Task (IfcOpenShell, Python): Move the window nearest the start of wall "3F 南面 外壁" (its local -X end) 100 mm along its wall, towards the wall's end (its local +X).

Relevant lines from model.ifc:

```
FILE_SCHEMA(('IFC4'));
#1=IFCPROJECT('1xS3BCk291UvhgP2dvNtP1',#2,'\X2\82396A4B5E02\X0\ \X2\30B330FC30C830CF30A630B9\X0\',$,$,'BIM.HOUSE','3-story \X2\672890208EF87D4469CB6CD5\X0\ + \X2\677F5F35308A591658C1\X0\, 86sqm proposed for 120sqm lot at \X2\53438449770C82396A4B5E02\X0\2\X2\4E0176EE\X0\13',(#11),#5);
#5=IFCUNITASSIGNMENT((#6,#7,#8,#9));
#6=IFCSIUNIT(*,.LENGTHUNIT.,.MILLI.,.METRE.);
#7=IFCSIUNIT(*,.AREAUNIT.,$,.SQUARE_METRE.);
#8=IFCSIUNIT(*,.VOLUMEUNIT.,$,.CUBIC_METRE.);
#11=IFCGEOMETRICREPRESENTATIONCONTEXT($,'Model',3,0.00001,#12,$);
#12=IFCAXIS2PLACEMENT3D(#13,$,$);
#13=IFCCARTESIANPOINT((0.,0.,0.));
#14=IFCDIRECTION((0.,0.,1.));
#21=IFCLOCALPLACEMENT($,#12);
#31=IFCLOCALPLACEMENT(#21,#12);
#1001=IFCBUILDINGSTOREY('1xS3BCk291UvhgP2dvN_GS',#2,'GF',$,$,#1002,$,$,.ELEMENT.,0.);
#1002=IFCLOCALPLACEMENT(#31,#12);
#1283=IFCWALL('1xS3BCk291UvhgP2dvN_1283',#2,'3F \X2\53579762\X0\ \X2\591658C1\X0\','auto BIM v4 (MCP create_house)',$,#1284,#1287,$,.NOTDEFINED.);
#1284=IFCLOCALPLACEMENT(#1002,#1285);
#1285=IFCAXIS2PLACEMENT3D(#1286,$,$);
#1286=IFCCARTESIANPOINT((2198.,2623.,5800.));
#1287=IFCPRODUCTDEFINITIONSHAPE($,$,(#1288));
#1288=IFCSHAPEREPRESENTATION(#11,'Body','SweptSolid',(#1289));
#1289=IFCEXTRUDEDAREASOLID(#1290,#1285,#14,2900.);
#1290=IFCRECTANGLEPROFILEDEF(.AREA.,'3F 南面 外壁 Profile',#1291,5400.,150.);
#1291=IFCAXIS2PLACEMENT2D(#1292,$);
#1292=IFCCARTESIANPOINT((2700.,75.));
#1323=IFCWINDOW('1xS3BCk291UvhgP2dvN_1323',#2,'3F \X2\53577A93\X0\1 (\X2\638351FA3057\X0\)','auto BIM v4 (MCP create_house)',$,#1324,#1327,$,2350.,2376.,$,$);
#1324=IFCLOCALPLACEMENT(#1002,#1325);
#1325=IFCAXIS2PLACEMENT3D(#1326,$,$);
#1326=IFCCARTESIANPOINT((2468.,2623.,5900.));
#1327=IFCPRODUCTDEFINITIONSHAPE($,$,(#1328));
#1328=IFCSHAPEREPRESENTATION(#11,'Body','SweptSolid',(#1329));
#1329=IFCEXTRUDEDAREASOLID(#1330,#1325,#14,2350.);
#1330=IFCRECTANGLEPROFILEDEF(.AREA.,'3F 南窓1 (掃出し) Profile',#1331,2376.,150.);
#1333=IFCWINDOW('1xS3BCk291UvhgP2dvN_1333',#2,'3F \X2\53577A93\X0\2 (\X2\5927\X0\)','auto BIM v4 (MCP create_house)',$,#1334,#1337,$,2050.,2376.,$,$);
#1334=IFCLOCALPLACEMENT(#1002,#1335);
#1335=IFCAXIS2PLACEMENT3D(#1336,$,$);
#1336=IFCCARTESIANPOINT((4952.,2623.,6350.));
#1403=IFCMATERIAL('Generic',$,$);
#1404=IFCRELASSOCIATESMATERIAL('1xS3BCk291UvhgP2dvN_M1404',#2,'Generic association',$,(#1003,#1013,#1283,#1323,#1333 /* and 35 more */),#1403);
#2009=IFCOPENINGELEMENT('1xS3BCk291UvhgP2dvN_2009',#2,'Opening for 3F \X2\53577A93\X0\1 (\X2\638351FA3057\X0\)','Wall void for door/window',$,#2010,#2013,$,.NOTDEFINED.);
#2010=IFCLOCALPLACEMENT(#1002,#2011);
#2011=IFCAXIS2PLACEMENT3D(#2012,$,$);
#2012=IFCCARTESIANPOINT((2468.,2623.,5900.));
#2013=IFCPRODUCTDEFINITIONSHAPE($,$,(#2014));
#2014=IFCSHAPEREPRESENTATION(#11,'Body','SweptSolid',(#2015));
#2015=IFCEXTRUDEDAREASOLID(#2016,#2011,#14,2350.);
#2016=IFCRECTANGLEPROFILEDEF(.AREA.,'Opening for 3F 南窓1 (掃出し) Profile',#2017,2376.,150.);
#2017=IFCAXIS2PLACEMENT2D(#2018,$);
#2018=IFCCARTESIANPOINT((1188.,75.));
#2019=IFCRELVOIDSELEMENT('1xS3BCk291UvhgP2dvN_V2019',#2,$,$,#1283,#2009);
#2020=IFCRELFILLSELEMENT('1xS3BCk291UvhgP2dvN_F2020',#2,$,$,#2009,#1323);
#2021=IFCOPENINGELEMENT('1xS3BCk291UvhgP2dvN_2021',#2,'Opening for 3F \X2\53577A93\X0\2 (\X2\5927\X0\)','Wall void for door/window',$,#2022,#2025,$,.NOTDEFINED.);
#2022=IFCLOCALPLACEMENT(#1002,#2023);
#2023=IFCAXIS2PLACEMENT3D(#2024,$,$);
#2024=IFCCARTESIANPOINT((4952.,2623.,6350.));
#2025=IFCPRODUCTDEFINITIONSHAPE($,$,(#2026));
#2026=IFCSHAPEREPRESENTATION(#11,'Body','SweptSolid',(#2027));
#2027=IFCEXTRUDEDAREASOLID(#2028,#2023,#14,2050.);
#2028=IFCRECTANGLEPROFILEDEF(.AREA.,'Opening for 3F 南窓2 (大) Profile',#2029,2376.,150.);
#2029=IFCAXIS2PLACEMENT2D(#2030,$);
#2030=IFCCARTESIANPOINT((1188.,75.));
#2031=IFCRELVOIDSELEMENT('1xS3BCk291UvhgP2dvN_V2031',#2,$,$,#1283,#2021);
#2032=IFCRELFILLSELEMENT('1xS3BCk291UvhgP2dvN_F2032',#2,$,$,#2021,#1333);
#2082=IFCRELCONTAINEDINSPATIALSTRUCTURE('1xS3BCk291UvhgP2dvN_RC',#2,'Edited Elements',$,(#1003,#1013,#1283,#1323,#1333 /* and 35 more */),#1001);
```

```python
import ifcopenshell
import ifcopenshell.api.geometry
import ifcopenshell.util.placement

model = ifcopenshell.open("model.ifc")

window = model.by_guid("1xS3BCk291UvhgP2dvN_1323")
opening = window.FillsVoids[0].RelatingOpeningElement
wall = opening.VoidsElements[0].RelatingBuildingElement

wall_matrix = ifcopenshell.util.placement.get_local_placement(wall.ObjectPlacement)
shift = wall_matrix[:3, 0] * 100.0
before = ifcopenshell.util.placement.get_local_placement(window.ObjectPlacement)[:3, 3].copy()

# The window is not placed relative to its opening, so move both.
for product in (opening, window):
    matrix = ifcopenshell.util.placement.get_local_placement(product.ObjectPlacement)
    matrix[:3, 3] += shift
    ifcopenshell.api.geometry.edit_object_placement(model, product=product, matrix=matrix, is_si=False)

after = ifcopenshell.util.placement.get_local_placement(window.ObjectPlacement)[:3, 3]
print("window moved by", (after - before).round(3) + 0.0)

model.write("model_v2.ifc")
```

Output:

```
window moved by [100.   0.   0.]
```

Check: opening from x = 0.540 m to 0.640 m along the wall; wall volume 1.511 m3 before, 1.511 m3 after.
